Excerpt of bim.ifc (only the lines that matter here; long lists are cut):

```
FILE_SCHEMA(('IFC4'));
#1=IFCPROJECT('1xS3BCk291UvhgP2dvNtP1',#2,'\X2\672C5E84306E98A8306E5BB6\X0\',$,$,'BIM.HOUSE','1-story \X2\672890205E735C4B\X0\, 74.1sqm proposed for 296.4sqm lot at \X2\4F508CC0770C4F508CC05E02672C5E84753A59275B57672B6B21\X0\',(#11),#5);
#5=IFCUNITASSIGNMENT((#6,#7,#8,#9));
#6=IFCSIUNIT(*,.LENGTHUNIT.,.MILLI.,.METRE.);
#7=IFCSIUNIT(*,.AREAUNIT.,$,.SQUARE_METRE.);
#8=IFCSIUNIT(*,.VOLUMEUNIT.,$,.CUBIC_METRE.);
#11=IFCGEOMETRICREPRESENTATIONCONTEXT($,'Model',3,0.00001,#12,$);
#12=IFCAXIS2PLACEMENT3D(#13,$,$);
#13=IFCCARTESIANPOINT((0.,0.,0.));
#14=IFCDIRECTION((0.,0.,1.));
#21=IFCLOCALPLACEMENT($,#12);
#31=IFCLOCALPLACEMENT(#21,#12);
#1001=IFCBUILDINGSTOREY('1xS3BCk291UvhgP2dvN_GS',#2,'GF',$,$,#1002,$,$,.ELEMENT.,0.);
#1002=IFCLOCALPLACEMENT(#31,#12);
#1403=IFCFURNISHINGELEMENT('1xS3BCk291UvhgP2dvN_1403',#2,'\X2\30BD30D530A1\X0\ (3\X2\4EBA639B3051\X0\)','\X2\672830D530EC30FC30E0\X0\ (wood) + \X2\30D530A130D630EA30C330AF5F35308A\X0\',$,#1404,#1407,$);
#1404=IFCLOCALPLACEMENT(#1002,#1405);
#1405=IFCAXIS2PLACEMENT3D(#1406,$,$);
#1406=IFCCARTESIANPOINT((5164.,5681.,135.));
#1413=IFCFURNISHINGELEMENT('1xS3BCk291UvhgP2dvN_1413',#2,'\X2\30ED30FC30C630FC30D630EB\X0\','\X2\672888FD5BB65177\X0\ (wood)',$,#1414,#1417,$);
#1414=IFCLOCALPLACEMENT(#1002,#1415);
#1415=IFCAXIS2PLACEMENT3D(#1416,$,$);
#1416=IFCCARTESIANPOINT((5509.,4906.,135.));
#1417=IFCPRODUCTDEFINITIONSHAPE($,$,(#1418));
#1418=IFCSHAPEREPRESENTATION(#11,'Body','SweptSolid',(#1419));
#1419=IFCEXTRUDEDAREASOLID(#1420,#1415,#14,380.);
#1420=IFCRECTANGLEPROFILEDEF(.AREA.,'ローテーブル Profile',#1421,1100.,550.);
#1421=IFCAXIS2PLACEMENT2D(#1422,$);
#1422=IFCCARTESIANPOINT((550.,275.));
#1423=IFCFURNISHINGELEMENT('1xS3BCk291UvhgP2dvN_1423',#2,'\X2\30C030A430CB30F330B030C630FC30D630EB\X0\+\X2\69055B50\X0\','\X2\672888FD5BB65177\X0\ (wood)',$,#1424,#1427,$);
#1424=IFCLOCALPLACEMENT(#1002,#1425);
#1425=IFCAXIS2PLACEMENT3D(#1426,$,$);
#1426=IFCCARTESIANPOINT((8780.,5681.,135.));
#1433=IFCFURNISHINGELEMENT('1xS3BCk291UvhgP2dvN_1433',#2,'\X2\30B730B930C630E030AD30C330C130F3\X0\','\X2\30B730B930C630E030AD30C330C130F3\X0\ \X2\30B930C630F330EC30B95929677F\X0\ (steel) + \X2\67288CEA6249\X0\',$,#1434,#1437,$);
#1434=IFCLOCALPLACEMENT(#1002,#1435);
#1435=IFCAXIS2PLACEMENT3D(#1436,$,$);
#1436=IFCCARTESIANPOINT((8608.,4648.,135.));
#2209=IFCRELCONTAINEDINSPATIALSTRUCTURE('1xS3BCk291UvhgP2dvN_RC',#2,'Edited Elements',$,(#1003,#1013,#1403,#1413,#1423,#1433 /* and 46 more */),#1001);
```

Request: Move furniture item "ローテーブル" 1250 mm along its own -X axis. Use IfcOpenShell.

```python
import ifcopenshell
import ifcopenshell.api.geometry
import ifcopenshell.util.placement
import ifcopenshell.util.unit

model = ifcopenshell.open("bim.ifc")
unit_scale = ifcopenshell.util.unit.calculate_unit_scale(model)

item = model.by_guid("1xS3BCk291UvhgP2dvN_1413")
matrix = ifcopenshell.util.placement.get_local_placement(item.ObjectPlacement)
matrix[:3, 3] -= matrix[:3, 0] * 1.25 / unit_scale
ifcopenshell.api.geometry.edit_object_placement(model, product=item, matrix=matrix, is_si=False)

print(ifcopenshell.util.placement.get_local_placement(item.ObjectPlacement).round(3) + 0.0)

model.write("bim-out.ifc")
```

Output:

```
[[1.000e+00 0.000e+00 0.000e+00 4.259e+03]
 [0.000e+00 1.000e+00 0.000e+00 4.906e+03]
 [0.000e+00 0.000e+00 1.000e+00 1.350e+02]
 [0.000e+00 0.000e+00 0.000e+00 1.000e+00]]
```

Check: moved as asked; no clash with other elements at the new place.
